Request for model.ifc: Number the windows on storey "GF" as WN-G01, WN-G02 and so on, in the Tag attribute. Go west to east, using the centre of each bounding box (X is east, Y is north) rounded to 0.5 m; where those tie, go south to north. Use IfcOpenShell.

First a look at what the model holds.

```python
import ifcopenshell
import ifcopenshell.util.element
import ifcopenshell.util.placement

model = ifcopenshell.open("model.ifc")
print(model.schema)
storey = next(s for s in model.by_type("IfcBuildingStorey") if s.Name == "GF")
windows = [e for e in ifcopenshell.util.element.get_decomposition(storey) if e.is_a("IfcWindow")]
for e in sorted(windows, key=lambda e: e.id()):
    origin = ifcopenshell.util.placement.get_local_placement(e.ObjectPlacement)[:3, 3]
    print(e.id(), e.Tag, e.Name, origin.round(2) + 0.0, sep=" | ")
```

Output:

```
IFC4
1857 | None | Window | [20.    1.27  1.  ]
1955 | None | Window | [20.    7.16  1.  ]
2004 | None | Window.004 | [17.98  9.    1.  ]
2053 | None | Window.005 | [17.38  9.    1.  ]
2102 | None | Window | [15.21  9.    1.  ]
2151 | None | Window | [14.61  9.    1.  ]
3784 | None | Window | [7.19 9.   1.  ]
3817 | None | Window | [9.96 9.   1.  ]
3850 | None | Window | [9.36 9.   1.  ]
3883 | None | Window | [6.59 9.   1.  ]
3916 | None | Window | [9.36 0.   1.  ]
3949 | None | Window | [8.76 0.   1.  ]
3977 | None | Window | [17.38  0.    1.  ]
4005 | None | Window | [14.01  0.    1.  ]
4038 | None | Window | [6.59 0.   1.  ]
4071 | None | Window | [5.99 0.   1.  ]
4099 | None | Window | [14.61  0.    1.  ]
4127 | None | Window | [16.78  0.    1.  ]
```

```python
import ifcopenshell
import ifcopenshell.geom
import ifcopenshell.util.element
import ifcopenshell.util.shape

model = ifcopenshell.open("model.ifc")
settings = ifcopenshell.geom.settings()
settings.set("use-world-coords", True)


def centre(element):
    shape = ifcopenshell.geom.create_shape(settings, element)
    return ifcopenshell.util.shape.get_bbox_centroid(shape.geometry)


storey = next(s for s in model.by_type("IfcBuildingStorey") if s.Name == "GF")
windows = [e for e in ifcopenshell.util.element.get_decomposition(storey) if e.is_a("IfcWindow")]

# Insertion points can sit at a corner or the storey origin, so sort by the geometry (in metres).
centres = {e: centre(e) for e in windows}
windows.sort(key=lambda e: (round(centres[e][0] / 0.5), centres[e][1]))

for i, e in enumerate(windows, start=1):
    number = f"WN-G{i:02d}"
    e.Tag = number
    print(e.id(), number)

model.write("model_edited.ifc")
```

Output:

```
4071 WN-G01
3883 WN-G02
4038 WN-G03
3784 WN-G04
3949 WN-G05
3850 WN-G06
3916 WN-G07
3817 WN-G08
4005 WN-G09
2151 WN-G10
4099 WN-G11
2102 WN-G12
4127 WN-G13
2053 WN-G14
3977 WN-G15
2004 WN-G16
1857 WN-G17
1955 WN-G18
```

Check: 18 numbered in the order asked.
